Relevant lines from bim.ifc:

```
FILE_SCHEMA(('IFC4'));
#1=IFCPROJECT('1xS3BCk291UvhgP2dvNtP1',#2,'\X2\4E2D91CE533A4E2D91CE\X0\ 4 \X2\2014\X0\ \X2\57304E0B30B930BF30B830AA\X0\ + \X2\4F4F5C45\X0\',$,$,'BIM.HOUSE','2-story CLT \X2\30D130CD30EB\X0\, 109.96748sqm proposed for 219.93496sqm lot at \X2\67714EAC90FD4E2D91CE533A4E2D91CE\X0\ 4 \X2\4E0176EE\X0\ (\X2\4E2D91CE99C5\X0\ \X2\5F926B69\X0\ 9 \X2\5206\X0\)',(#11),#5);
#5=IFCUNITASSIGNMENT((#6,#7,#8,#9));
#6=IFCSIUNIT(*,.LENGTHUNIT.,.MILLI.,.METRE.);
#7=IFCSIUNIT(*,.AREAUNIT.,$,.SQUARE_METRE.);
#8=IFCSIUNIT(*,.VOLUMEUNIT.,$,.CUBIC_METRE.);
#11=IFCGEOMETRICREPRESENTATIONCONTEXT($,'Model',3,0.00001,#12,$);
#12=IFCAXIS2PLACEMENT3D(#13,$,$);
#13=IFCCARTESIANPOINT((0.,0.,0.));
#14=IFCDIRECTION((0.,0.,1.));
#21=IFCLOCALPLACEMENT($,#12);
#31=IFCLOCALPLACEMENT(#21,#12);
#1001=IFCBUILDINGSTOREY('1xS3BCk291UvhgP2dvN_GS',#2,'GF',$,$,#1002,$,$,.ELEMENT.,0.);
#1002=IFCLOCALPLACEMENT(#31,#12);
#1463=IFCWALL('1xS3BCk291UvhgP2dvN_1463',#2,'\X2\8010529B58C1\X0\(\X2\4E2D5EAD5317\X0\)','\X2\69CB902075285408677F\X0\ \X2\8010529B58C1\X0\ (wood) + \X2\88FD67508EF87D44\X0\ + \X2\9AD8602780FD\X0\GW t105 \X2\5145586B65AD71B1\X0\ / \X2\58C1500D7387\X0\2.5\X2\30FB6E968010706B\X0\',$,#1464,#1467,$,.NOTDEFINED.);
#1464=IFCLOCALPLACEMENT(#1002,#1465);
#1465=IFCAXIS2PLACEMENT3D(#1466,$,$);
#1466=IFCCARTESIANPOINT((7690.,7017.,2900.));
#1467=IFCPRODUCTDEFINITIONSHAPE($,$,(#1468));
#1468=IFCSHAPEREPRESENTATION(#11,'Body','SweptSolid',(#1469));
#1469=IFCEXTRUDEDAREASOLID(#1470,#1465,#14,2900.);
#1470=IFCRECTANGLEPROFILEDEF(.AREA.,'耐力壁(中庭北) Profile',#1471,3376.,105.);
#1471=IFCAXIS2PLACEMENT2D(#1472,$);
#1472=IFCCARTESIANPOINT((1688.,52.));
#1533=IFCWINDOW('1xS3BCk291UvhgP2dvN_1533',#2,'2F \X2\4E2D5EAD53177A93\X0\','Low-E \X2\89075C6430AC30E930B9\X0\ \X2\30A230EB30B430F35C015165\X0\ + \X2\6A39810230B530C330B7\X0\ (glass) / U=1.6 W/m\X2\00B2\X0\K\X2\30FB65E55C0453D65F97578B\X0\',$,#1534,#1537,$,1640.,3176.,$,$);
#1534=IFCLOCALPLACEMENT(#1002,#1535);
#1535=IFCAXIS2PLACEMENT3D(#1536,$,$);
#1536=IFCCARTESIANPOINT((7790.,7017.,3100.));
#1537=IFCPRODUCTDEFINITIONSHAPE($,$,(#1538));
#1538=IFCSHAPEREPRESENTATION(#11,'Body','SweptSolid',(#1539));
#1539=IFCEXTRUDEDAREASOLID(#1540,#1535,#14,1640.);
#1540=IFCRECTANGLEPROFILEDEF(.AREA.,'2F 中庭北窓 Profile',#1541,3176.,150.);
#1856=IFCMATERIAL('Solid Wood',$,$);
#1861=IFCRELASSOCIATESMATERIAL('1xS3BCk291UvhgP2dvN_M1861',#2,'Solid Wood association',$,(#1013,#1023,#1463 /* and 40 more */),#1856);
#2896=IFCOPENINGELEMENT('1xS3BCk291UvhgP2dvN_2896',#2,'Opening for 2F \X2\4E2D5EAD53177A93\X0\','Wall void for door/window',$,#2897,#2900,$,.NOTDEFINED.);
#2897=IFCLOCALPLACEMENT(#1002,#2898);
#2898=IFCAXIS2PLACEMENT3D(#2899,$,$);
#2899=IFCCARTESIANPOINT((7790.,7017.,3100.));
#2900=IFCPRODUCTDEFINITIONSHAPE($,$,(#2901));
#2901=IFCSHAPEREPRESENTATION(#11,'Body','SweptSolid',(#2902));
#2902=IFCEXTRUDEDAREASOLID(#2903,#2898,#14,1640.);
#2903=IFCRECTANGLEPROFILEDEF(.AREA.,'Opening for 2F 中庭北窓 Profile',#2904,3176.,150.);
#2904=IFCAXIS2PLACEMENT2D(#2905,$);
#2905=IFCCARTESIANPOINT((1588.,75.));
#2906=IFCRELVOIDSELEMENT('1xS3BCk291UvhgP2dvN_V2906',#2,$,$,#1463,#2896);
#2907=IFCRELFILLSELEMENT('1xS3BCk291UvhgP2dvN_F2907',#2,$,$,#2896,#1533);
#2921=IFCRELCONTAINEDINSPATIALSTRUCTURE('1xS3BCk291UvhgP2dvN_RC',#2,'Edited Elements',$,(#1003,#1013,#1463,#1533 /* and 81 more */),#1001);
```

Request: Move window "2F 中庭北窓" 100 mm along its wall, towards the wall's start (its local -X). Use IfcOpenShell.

```python
import ifcopenshell
import ifcopenshell.api.geometry
import ifcopenshell.util.placement
import ifcopenshell.util.unit

model = ifcopenshell.open("bim.ifc")
unit_scale = ifcopenshell.util.unit.calculate_unit_scale(model)

window = model.by_id(1533)
opening = window.FillsVoids[0].RelatingOpeningElement
wall = opening.VoidsElements[0].RelatingBuildingElement

wall_matrix = ifcopenshell.util.placement.get_local_placement(wall.ObjectPlacement)
shift = wall_matrix[:3, 0] * -0.1 / unit_scale
before = ifcopenshell.util.placement.get_local_placement(window.ObjectPlacement)[:3, 3].copy()

# The window is not placed relative to its opening, so move both.
for product in (opening, window):
    matrix = ifcopenshell.util.placement.get_local_placement(product.ObjectPlacement)
    matrix[:3, 3] += shift
    ifcopenshell.api.geometry.edit_object_placement(model, product=product, matrix=matrix, is_si=False)

after = ifcopenshell.util.placement.get_local_placement(window.ObjectPlacement)[:3, 3]
print("window moved by", (after - before).round(3) + 0.0)

model.write("bim_edited.ifc")
```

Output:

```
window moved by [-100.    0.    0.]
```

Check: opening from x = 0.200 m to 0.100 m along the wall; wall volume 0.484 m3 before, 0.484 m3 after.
